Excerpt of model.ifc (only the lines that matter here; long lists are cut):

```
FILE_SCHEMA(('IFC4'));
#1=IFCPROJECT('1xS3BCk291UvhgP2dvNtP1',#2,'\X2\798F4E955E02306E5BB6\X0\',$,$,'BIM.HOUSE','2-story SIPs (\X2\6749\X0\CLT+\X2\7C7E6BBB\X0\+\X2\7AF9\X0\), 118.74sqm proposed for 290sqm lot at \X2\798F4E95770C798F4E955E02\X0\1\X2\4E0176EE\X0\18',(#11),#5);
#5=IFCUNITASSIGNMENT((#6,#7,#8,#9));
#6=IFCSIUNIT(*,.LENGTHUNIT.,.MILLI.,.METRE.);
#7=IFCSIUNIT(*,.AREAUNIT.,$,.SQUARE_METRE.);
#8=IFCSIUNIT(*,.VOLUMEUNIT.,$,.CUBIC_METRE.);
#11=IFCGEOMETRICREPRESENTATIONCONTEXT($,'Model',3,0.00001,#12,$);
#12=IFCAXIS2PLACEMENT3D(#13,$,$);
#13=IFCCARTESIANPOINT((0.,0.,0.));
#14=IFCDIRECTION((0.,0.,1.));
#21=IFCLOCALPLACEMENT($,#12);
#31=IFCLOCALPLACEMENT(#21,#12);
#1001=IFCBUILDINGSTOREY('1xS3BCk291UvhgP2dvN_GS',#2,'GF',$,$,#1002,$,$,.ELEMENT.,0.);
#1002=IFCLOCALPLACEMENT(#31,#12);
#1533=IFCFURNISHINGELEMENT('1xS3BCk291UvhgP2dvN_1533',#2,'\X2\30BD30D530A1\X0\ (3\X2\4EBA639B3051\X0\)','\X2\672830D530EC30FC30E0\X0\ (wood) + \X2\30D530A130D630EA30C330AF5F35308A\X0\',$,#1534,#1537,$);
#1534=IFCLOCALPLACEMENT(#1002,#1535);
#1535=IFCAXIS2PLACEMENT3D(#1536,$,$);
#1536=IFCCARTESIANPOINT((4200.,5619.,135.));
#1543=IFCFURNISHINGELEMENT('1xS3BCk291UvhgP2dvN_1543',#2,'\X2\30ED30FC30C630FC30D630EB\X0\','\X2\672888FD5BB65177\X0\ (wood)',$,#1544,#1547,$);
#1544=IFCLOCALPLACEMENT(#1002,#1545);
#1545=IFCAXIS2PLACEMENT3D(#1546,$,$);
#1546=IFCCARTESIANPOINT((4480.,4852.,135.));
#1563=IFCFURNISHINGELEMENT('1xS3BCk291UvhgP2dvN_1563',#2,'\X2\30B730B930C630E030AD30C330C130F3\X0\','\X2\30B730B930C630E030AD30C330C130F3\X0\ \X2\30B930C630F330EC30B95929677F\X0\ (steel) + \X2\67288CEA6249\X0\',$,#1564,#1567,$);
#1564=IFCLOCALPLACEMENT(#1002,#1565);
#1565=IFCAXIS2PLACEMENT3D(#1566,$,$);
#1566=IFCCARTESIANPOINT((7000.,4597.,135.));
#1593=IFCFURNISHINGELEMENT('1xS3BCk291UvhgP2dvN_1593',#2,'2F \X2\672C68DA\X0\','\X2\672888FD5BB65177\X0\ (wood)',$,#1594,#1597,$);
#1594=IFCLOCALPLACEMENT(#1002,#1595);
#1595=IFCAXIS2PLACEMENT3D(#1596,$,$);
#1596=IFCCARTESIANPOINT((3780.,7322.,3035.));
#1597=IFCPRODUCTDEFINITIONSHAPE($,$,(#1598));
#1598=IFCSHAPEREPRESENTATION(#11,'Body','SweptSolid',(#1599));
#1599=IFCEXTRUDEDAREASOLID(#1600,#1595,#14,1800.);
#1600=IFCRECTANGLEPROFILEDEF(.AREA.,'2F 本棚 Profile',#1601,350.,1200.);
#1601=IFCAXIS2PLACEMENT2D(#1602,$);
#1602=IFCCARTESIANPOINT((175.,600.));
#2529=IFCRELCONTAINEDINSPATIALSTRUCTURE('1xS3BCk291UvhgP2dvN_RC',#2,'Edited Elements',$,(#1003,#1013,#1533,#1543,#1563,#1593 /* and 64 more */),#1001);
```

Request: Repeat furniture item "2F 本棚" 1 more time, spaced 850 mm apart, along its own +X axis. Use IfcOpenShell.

```python
import ifcopenshell
import ifcopenshell.api.geometry
import ifcopenshell.api.root
import ifcopenshell.util.element
import ifcopenshell.util.placement
import ifcopenshell.util.unit

model = ifcopenshell.open("model.ifc")
unit_scale = ifcopenshell.util.unit.calculate_unit_scale(model)


def reuse_history(source, copy):
    """copy_class also copies each property set's owner history, people and application; keep the originals."""
    for rel in copy.IsDefinedBy:
        if rel.is_a("IfcRelDefinesByProperties") and (history := rel.RelatingPropertyDefinition.OwnerHistory):
            rel.RelatingPropertyDefinition.OwnerHistory = source.OwnerHistory
            ifcopenshell.util.element.remove_deep2(model, history)


source = model.by_id(1593)
base = ifcopenshell.util.placement.get_local_placement(source.ObjectPlacement)
step = base[:3, 0] * 0.85 / unit_scale

for i in range(1, 2):
    copy = ifcopenshell.api.root.copy_class(model, product=source)
    copy.Representation = ifcopenshell.util.element.copy_deep(
        model, source.Representation, exclude=["IfcGeometricRepresentationContext", "IfcRepresentationMap"]
    )
    reuse_history(source, copy)
    matrix = base.copy()
    matrix[:3, 3] += i * step
    print("added at", matrix[:3, 3].round(3) + 0.0)
    ifcopenshell.api.geometry.edit_object_placement(model, product=copy, matrix=matrix, is_si=False)

model.write("model_edited.ifc")
```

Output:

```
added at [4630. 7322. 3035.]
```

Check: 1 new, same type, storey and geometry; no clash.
